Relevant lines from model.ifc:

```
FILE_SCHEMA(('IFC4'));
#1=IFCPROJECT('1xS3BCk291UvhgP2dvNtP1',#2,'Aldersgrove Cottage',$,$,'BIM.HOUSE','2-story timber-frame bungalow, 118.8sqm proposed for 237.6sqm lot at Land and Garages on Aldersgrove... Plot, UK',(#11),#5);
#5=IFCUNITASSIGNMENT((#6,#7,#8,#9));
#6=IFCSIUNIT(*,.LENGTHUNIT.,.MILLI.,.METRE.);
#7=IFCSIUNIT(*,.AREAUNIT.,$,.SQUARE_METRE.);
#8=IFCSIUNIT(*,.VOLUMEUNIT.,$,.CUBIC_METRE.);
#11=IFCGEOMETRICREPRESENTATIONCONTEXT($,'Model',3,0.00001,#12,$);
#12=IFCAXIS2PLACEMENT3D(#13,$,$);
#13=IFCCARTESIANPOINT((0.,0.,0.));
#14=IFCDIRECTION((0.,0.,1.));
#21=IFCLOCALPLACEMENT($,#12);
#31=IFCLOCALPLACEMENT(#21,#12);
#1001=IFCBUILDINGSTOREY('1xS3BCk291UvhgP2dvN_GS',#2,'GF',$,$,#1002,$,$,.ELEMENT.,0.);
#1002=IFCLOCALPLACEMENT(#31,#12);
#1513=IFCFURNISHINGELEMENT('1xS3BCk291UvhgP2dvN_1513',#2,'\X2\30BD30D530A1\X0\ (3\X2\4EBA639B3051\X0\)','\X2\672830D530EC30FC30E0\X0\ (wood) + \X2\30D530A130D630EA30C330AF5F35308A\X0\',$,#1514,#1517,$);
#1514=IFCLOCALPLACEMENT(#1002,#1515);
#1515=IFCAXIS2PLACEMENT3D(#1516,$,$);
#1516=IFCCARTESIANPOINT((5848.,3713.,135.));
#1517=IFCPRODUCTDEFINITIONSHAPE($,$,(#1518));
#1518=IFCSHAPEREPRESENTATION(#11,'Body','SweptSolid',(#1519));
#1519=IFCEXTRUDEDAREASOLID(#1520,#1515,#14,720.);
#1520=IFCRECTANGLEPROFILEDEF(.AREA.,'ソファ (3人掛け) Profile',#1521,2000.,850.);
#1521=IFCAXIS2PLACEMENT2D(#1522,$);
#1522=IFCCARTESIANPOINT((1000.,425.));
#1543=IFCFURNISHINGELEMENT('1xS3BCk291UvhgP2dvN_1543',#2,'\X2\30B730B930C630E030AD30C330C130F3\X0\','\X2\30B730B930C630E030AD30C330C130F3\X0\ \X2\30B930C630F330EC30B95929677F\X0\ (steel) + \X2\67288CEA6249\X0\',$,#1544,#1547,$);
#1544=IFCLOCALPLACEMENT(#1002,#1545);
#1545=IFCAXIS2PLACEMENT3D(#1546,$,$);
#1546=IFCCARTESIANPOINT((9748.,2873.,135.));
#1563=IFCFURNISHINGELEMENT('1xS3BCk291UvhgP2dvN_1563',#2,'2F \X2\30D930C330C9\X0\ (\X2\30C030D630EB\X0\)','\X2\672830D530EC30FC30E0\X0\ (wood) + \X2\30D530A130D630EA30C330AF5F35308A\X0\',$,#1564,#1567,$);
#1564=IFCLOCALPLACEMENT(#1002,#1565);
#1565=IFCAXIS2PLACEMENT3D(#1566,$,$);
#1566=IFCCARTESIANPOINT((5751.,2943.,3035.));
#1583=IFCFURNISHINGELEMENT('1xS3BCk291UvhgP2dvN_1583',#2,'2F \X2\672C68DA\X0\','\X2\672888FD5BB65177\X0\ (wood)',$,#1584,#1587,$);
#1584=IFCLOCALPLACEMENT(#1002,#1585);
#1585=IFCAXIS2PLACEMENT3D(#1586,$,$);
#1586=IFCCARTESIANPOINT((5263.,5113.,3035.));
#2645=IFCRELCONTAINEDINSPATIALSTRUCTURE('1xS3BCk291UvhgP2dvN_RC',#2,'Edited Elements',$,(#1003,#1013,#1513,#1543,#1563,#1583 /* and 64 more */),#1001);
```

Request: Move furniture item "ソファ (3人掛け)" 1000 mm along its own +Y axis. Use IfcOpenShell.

```python
import ifcopenshell
import ifcopenshell.api.geometry
import ifcopenshell.util.placement

model = ifcopenshell.open("model.ifc")

item = model.by_guid("1xS3BCk291UvhgP2dvN_1513")
matrix = ifcopenshell.util.placement.get_local_placement(item.ObjectPlacement)
matrix[:3, 3] += matrix[:3, 1] * 1000.0
ifcopenshell.api.geometry.edit_object_placement(model, product=item, matrix=matrix, is_si=False)

print(ifcopenshell.util.placement.get_local_placement(item.ObjectPlacement).round(3) + 0.0)

model.write("model-out.ifc")
```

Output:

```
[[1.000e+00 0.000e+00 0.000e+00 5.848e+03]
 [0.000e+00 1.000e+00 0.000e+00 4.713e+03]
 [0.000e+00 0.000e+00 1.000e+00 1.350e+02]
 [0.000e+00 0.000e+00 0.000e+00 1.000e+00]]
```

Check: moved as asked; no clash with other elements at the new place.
